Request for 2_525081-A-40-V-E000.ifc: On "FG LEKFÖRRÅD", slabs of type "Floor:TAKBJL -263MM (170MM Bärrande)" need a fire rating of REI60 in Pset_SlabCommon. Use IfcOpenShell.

First a look at what the model holds.

```python
import ifcopenshell
import ifcopenshell.util.element

model = ifcopenshell.open("2_525081-A-40-V-E000.ifc")
print(model.schema)
storey = next(s for s in model.by_type("IfcBuildingStorey") if s.Name == "FG LEKFÖRRÅD")
slabs = [e for e in ifcopenshell.util.element.get_decomposition(storey) if e.is_a("IfcSlab")]
seen = {}
for e in slabs:
    element_type = ifcopenshell.util.element.get_type(e)
    key = (element_type.Name if element_type != e and element_type else None, ifcopenshell.util.element.get_pset(e, "Pset_SlabCommon", "FireRating"))
    seen[key] = seen.get(key, 0) + 1
for (name, value), count in sorted(seen.items(), key=str):
    print(count, "x", name, "|", value)
```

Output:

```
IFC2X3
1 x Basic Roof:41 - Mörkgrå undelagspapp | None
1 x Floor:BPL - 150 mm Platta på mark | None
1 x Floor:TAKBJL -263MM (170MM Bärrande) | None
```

```python
import ifcopenshell
import ifcopenshell.api.pset
import ifcopenshell.util.element

model = ifcopenshell.open("2_525081-A-40-V-E000.ifc")

storey = next(s for s in model.by_type("IfcBuildingStorey") if s.Name == "FG LEKFÖRRÅD")
slabs = [e for e in ifcopenshell.util.element.get_decomposition(storey) if e.is_a("IfcSlab")]

count = 0
for e in slabs:
    element_type = ifcopenshell.util.element.get_type(e)
    if element_type in (None, e) or element_type.Name != "Floor:TAKBJL -263MM (170MM Bärrande)":
        continue
    # add_pset returns the element's existing set when there is one.
    pset = ifcopenshell.api.pset.add_pset(model, product=e, name="Pset_SlabCommon")
    ifcopenshell.api.pset.edit_pset(model, pset=pset, properties={"FireRating": "REI60"})
    count += 1

print(count, "slabs updated")

model.write("2_525081-A-40-V-E000_rev.ifc")
```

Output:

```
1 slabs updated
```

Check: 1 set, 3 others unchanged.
